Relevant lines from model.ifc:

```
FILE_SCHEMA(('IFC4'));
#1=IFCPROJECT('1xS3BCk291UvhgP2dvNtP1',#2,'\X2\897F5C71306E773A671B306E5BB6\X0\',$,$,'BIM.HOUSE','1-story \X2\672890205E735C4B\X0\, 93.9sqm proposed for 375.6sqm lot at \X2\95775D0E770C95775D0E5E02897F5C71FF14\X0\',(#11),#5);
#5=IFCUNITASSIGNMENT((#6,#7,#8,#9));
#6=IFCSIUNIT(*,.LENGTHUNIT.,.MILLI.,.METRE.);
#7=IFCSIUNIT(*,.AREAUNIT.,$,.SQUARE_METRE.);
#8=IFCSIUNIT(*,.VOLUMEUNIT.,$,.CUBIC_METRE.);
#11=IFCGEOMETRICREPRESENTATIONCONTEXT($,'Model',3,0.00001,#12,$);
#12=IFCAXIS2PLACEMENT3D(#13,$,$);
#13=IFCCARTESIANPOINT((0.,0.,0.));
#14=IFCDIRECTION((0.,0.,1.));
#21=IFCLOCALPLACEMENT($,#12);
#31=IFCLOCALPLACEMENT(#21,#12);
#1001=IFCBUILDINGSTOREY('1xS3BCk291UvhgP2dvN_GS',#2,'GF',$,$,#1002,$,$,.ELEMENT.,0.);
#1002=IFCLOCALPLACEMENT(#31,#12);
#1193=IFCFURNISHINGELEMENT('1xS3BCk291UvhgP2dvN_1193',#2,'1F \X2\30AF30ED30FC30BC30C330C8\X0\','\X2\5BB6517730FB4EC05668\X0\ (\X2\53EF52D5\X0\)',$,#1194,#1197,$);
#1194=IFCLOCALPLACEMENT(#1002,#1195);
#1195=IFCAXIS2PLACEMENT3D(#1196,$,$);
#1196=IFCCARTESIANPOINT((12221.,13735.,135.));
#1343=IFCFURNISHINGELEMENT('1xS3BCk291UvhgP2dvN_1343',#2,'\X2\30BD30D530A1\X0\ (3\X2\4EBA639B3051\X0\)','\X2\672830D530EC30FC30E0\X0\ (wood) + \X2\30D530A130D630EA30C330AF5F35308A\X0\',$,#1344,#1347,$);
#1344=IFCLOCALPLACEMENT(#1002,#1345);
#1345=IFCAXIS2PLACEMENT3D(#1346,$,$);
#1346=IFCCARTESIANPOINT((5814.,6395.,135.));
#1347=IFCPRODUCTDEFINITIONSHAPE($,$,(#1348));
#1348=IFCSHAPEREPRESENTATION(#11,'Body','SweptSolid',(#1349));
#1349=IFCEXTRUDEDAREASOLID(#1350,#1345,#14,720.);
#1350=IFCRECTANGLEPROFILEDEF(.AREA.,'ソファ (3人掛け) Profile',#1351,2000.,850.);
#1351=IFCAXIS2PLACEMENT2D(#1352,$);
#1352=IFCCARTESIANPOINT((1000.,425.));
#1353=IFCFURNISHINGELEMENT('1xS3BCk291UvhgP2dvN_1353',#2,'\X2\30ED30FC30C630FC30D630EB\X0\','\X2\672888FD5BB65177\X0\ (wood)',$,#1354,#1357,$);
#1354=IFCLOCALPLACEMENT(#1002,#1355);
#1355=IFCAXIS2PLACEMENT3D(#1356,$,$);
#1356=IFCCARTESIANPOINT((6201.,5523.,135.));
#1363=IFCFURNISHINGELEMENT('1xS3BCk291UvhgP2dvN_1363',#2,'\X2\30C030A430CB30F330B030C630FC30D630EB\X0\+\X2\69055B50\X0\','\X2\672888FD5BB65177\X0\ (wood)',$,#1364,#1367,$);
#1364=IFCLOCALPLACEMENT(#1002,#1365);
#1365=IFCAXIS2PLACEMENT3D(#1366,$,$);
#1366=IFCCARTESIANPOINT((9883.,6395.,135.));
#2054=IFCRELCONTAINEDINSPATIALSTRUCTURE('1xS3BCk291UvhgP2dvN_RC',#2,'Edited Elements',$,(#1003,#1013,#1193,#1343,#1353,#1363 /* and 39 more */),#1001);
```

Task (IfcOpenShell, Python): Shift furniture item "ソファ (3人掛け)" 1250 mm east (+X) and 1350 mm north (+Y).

```python
import ifcopenshell
import ifcopenshell.api.geometry
import ifcopenshell.util.placement
import ifcopenshell.util.unit

model = ifcopenshell.open("model.ifc")
unit_scale = ifcopenshell.util.unit.calculate_unit_scale(model)

item = model.by_id(1343)
matrix = ifcopenshell.util.placement.get_local_placement(item.ObjectPlacement)
matrix[0, 3] += 1.25 / unit_scale
matrix[1, 3] += 1.35 / unit_scale
ifcopenshell.api.geometry.edit_object_placement(model, product=item, matrix=matrix, is_si=False)

print(ifcopenshell.util.placement.get_local_placement(item.ObjectPlacement).round(3) + 0.0)

model.write("model_v2.ifc")
```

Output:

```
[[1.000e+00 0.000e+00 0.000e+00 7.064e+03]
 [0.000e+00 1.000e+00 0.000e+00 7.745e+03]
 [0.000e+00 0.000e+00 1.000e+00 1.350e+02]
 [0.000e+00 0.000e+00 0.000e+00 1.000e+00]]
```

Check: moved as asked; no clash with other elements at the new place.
